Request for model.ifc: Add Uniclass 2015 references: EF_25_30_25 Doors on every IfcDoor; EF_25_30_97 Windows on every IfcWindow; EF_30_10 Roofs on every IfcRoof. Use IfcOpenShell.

First a look at what the model holds.

```python
import ifcopenshell

model = ifcopenshell.open("model.ifc")
print(model.schema)
print("classifications:", [c.Name for c in model.by_type("IfcClassification")])
for ifc_class in ("IfcDoor", "IfcRoof", "IfcStair", "IfcWall", "IfcWindow"):
    print(ifc_class, len(model.by_type(ifc_class)))
```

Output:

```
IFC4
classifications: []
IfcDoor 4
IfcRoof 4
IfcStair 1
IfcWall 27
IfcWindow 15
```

```python
import ifcopenshell
import ifcopenshell.api.classification

model = ifcopenshell.open("model.ifc")

system = ifcopenshell.api.classification.add_classification(model, classification="Uniclass 2015")

codes = {
    "IfcDoor": ("EF_25_30_25", "Doors"),
    "IfcWindow": ("EF_25_30_97", "Windows"),
    "IfcRoof": ("EF_30_10", "Roofs"),
}
for ifc_class, (code, name) in codes.items():
    products = model.by_type(ifc_class)
    ifcopenshell.api.classification.add_reference(
        model, products=products, classification=system, identification=code, name=name
    )
    print(code, len(products))

model.write("model_updated.ifc")
```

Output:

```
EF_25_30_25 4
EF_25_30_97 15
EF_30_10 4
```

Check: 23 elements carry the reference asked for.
